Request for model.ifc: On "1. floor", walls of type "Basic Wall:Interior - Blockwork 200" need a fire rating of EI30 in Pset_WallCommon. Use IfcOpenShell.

First a look at what the model holds.

```python
import ifcopenshell
import ifcopenshell.util.element

model = ifcopenshell.open("model.ifc")
print(model.schema)
storey = next(s for s in model.by_type("IfcBuildingStorey") if s.Name == "1. floor")
walls = [e for e in ifcopenshell.util.element.get_decomposition(storey) if e.is_a("IfcWall")]
seen = {}
for e in walls:
    element_type = ifcopenshell.util.element.get_type(e)
    key = (element_type.Name if element_type != e and element_type else None, ifcopenshell.util.element.get_pset(e, "Pset_WallCommon", "FireRating"))
    seen[key] = seen.get(key, 0) + 1
for (name, value), count in sorted(seen.items(), key=str):
    print(count, "x", name, "|", value)
```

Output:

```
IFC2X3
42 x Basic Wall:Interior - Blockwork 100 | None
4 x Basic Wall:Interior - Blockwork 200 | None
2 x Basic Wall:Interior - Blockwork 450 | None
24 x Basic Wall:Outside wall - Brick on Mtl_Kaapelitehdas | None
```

```python
import ifcopenshell
import ifcopenshell.api.pset
import ifcopenshell.util.element

model = ifcopenshell.open("model.ifc")

storey = next(s for s in model.by_type("IfcBuildingStorey") if s.Name == "1. floor")
walls = [e for e in ifcopenshell.util.element.get_decomposition(storey) if e.is_a("IfcWall")]

count = 0
for e in walls:
    element_type = ifcopenshell.util.element.get_type(e)
    if element_type in (None, e) or element_type.Name != "Basic Wall:Interior - Blockwork 200":
        continue
    # add_pset returns the element's existing set when there is one.
    pset = ifcopenshell.api.pset.add_pset(model, product=e, name="Pset_WallCommon")
    ifcopenshell.api.pset.edit_pset(model, pset=pset, properties={"FireRating": "EI30"})
    count += 1

print(count, "walls updated")

model.write("model_rev.ifc")
```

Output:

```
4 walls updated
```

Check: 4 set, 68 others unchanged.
